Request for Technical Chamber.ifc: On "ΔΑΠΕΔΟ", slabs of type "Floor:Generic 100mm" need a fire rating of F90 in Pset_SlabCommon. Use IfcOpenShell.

First a look at what the model holds.

```python
import ifcopenshell
import ifcopenshell.util.element

model = ifcopenshell.open("Technical Chamber.ifc")
print(model.schema)
storey = next(s for s in model.by_type("IfcBuildingStorey") if s.Name == "ΔΑΠΕΔΟ")
slabs = [e for e in ifcopenshell.util.element.get_decomposition(storey) if e.is_a("IfcSlab")]
seen = {}
for e in slabs:
    element_type = ifcopenshell.util.element.get_type(e)
    key = (element_type.Name if element_type != e and element_type else None, ifcopenshell.util.element.get_pset(e, "Pset_SlabCommon", "FireRating"))
    seen[key] = seen.get(key, 0) + 1
for (name, value), count in sorted(seen.items(), key=str):
    print(count, "x", name, "|", value)
```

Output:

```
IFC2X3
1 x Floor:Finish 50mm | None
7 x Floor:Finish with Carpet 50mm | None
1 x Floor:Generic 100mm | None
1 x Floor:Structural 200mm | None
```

```python
import ifcopenshell
import ifcopenshell.api.pset
import ifcopenshell.util.element

model = ifcopenshell.open("Technical Chamber.ifc")

storey = next(s for s in model.by_type("IfcBuildingStorey") if s.Name == "ΔΑΠΕΔΟ")
slabs = [e for e in ifcopenshell.util.element.get_decomposition(storey) if e.is_a("IfcSlab")]

count = 0
for e in slabs:
    element_type = ifcopenshell.util.element.get_type(e)
    if element_type in (None, e) or element_type.Name != "Floor:Generic 100mm":
        continue
    # add_pset returns the element's existing set when there is one.
    pset = ifcopenshell.api.pset.add_pset(model, product=e, name="Pset_SlabCommon")
    ifcopenshell.api.pset.edit_pset(model, pset=pset, properties={"FireRating": "F90"})
    count += 1

print(count, "slabs updated")

model.write("Technical Chamber_v2.ifc")
```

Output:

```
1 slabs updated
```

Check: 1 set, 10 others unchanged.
